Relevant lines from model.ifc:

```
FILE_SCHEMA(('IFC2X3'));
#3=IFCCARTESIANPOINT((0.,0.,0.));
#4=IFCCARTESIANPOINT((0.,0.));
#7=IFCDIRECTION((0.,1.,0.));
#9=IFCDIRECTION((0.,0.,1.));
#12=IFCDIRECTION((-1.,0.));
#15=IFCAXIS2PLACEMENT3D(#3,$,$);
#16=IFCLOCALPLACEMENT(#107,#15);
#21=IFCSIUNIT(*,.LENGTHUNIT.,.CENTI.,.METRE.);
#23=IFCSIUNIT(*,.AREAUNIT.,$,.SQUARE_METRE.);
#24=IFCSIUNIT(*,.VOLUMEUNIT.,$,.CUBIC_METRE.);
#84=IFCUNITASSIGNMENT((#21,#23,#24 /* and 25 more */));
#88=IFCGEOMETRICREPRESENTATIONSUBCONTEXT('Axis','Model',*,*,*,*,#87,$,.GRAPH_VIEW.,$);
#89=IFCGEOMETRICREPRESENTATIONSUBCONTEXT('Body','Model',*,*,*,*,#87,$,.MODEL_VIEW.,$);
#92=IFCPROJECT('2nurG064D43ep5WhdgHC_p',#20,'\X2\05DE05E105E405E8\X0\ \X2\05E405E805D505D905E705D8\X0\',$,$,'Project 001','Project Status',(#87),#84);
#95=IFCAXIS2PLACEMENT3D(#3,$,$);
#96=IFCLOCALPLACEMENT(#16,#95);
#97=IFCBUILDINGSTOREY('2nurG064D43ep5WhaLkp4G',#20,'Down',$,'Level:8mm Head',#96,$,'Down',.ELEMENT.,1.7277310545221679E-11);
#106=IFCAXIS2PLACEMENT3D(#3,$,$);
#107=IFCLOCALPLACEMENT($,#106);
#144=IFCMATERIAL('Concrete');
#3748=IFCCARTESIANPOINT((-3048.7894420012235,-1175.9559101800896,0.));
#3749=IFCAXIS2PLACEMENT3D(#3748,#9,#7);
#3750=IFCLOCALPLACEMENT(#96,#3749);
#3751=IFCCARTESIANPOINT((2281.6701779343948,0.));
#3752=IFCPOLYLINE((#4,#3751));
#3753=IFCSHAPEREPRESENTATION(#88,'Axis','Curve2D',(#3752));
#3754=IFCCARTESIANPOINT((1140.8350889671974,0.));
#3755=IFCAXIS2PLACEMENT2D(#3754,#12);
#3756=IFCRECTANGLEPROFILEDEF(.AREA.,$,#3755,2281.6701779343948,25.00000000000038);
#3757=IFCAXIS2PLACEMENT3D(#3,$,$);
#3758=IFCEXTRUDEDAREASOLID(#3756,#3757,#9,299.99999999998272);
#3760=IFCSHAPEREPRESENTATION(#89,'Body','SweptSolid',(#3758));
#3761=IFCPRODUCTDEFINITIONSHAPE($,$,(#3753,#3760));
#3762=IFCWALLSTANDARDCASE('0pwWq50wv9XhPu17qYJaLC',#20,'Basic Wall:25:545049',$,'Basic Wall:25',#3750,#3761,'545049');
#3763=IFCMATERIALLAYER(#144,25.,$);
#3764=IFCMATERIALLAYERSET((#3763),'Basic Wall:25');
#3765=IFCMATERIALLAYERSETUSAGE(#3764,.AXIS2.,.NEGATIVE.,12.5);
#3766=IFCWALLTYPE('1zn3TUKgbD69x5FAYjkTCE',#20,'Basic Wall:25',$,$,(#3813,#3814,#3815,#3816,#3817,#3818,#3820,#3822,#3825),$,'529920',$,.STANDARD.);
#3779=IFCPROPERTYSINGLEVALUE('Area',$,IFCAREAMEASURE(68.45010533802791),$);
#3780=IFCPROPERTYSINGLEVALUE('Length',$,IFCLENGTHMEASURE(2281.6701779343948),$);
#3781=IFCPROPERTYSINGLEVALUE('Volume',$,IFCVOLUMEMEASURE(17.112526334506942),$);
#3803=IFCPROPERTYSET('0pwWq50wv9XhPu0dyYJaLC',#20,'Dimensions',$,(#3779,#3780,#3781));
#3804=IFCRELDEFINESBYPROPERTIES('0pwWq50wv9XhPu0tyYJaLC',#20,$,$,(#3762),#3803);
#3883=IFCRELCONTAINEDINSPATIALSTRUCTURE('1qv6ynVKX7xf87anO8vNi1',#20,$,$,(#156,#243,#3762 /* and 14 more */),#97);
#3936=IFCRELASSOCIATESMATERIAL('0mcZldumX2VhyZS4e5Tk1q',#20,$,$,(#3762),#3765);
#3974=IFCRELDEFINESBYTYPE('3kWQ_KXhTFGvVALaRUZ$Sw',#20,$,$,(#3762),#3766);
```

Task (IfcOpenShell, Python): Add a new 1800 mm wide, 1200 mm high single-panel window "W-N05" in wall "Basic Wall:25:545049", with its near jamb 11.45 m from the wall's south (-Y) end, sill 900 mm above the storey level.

```python
import numpy as np
import ifcopenshell
import ifcopenshell.api.feature
import ifcopenshell.api.geometry
import ifcopenshell.api.pset
import ifcopenshell.api.root
import ifcopenshell.api.spatial
import ifcopenshell.api.type
import ifcopenshell.geom
import ifcopenshell.util.element
import ifcopenshell.util.placement
import ifcopenshell.util.representation
import ifcopenshell.util.shape
import ifcopenshell.util.unit

model = ifcopenshell.open("model.ifc")
unit_scale = ifcopenshell.util.unit.calculate_unit_scale(model)
area_scale = ifcopenshell.util.unit.calculate_unit_scale(model, "AREAUNIT")
volume_scale = ifcopenshell.util.unit.calculate_unit_scale(model, "VOLUMEUNIT")
settings = ifcopenshell.geom.settings()


def volume(element):
    """Net volume in cubic metres, openings subtracted."""
    shape = ifcopenshell.geom.create_shape(settings, element)
    return ifcopenshell.util.shape.get_volume(shape.geometry)


wall = model.by_id(3762)
storey = ifcopenshell.util.element.get_container(wall, ifc_class="IfcBuildingStorey")
context = ifcopenshell.util.representation.get_context(model, "Model", "Body", "MODEL_VIEW")
before = volume(wall)

width, height, from_end, sill = 1.8, 1.2, 11.45, 0.9  # metres

# The wall runs along its own X axis, and the end named is its -X end.
wall_shape = ifcopenshell.geom.create_shape(settings, wall)
x, y, z = ifcopenshell.util.shape.get_vertices(wall_shape.geometry).T
start = x.min() + from_end
face, thickness = float(y.min()), float(y.max() - y.min())
wall_matrix = ifcopenshell.util.placement.get_local_placement(wall.ObjectPlacement)
level = ifcopenshell.util.placement.get_local_placement(storey.ObjectPlacement)[2, 3]


def in_wall(x, y):
    """Placement at x, y metres in the wall's axes, at sill height."""
    matrix = wall_matrix.copy()
    matrix[:, 3] = wall_matrix @ np.array([x / unit_scale, y / unit_scale, 0.0, 1.0])
    matrix[2, 3] = level + sill / unit_scale
    return matrix


# Opening: a box that overshoots both wall faces by 50 mm.
opening = ifcopenshell.api.root.create_entity(model, ifc_class="IfcOpeningElement")
box = ifcopenshell.api.geometry.add_wall_representation(
    model, context=context, length=width, height=height, thickness=thickness + 0.1
)
ifcopenshell.api.geometry.assign_representation(model, product=opening, representation=box)
ifcopenshell.api.geometry.edit_object_placement(model, product=opening, matrix=in_wall(start, face - 0.05), is_si=False)
ifcopenshell.api.feature.add_feature(model, feature=opening, element=wall)

window = ifcopenshell.api.root.create_entity(model, ifc_class="IfcWindow", name="W-N05")
window.OverallWidth, window.OverallHeight = width / unit_scale, height / unit_scale
body = ifcopenshell.api.geometry.add_window_representation(
    model,
    context=context,
    overall_width=window.OverallWidth,
    overall_height=window.OverallHeight,
    partition_type="SINGLE_PANEL",
)
ifcopenshell.api.geometry.assign_representation(model, product=window, representation=body)
ifcopenshell.api.spatial.assign_container(model, products=[window], relating_structure=storey)
fills = ifcopenshell.api.feature.add_filling(model, opening=opening, element=window)
fills.OwnerHistory = window.OwnerHistory  # required in IFC2X3

# IFC2X3 keeps the operation on the window style.
style = ifcopenshell.api.root.create_entity(model, ifc_class="IfcWindowStyle", name="W-N05")
style.OperationType, style.ConstructionType = "SINGLE_PANEL", "NOTDEFINED"
style.ParameterTakesPrecedence = style.Sizeable = False
ifcopenshell.api.type.assign_type(model, related_objects=[window], relating_type=style)

# Centre the window in the wall's thickness.
ifcopenshell.api.geometry.edit_object_placement(model, product=window, matrix=in_wall(start, face), is_si=False)
window_shape = ifcopenshell.geom.create_shape(settings, window)
depth = ifcopenshell.util.shape.get_vertices(window_shape.geometry)[:, 1]
offset = face + thickness / 2 - (depth.min() + depth.max()) / 2
ifcopenshell.api.geometry.edit_object_placement(model, product=window, matrix=in_wall(start, offset), is_si=False)

after = volume(wall)

# Update the wall's stored quantities.
pset = model.by_id(ifcopenshell.util.element.get_pset(wall, "Dimensions", should_inherit=False)["id"])
ifcopenshell.api.pset.edit_pset(model, pset=pset, properties={
    "Area": model.create_entity("IfcAreaMeasure", after / thickness / area_scale),
    "Volume": model.create_entity("IfcVolumeMeasure", after / volume_scale),
})

print(f"wall volume {before:.3f} -> {after:.3f} m3")

model.write("model_edited.ifc")
```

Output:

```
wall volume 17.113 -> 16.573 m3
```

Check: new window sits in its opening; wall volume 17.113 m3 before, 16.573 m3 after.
